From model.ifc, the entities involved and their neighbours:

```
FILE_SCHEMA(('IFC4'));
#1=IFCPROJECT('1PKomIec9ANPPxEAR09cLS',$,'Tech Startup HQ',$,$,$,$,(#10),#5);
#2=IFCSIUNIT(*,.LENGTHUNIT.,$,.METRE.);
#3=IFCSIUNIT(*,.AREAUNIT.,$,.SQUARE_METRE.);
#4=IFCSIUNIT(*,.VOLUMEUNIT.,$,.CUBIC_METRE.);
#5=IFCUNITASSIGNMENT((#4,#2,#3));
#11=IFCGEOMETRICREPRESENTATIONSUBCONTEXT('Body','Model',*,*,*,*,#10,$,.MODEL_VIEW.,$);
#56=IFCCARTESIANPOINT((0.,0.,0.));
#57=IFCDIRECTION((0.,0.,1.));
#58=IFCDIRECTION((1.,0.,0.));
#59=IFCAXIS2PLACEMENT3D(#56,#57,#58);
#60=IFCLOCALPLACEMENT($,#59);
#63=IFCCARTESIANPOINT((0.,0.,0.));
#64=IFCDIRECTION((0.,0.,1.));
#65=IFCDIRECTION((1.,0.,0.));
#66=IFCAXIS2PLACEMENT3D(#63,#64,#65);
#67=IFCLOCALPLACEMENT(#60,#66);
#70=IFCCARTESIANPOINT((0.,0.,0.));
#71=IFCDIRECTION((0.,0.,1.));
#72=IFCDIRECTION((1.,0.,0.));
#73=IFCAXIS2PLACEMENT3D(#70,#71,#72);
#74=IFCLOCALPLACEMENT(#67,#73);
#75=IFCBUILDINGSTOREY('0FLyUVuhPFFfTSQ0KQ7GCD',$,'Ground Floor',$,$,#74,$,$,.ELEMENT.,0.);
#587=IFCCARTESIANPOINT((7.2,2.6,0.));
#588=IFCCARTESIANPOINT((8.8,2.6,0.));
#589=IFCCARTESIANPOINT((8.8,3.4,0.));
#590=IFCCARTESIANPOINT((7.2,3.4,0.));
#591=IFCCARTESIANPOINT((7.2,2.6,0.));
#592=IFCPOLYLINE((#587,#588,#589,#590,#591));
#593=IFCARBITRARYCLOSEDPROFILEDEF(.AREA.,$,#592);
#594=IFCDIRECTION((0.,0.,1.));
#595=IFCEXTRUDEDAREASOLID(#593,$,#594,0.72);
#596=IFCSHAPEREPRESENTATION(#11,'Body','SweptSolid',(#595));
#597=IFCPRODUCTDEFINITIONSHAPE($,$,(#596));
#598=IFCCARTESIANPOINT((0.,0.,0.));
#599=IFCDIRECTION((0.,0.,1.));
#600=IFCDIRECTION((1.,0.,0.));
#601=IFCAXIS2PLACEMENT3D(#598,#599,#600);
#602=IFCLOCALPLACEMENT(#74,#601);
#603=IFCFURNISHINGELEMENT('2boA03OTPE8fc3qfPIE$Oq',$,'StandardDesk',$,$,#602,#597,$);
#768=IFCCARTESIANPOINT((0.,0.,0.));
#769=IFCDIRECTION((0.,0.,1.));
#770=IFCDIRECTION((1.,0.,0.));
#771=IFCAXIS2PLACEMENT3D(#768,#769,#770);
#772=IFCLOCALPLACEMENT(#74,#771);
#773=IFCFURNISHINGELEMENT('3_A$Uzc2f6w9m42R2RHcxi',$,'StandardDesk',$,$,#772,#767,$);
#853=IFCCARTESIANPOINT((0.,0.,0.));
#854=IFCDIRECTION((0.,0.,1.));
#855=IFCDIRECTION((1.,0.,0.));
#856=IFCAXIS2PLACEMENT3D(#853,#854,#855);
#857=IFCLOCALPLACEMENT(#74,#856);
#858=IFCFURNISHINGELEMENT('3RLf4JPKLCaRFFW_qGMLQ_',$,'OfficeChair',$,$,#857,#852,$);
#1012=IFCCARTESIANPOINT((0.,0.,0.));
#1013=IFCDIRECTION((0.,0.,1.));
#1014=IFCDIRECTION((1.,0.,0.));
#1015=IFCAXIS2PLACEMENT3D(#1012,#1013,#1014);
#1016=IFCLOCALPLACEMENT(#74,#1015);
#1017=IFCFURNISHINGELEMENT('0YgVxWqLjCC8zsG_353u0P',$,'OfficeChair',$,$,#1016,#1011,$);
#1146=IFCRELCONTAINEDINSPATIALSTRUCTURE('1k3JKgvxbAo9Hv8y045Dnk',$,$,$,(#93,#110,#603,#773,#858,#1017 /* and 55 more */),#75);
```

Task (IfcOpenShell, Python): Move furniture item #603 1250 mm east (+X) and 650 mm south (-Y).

```python
import ifcopenshell
import ifcopenshell.api.geometry
import ifcopenshell.util.placement

model = ifcopenshell.open("model.ifc")

item = model.by_guid("2boA03OTPE8fc3qfPIE$Oq")
matrix = ifcopenshell.util.placement.get_local_placement(item.ObjectPlacement)
matrix[0, 3] += 1.25
matrix[1, 3] -= 0.65
ifcopenshell.api.geometry.edit_object_placement(model, product=item, matrix=matrix, is_si=False)

print(ifcopenshell.util.placement.get_local_placement(item.ObjectPlacement).round(3) + 0.0)

model.write("model_rev.ifc")
```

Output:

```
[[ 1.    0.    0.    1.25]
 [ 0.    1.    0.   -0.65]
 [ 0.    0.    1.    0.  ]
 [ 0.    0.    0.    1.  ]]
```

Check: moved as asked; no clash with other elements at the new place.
